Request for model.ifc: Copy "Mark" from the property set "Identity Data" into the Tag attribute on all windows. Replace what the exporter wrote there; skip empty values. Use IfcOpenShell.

First a look at what the model holds.

```python
import ifcopenshell
import ifcopenshell.util.element

model = ifcopenshell.open("model.ifc")
print(model.schema)
windows = model.by_type("IfcWindow")
print(len(windows), "windows")
for e in windows[:8]:
    source = ifcopenshell.util.element.get_pset(e, "Identity Data", "Mark")
    target = e.Tag
    print(e.id(), repr(source), repr(target), sep=" | ")
```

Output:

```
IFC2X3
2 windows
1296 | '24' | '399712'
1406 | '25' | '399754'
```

```python
import ifcopenshell
import ifcopenshell.util.element

model = ifcopenshell.open("model.ifc")

count = 0
for e in model.by_type("IfcWindow"):
    value = ifcopenshell.util.element.get_pset(e, "Identity Data", "Mark")
    current = e.Tag
    if not value or not value.strip() or current == value:
        continue
    e.Tag = value
    count += 1

print(count, "windows updated")

model.write("model-out.ifc")
```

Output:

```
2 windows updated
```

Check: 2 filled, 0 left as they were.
